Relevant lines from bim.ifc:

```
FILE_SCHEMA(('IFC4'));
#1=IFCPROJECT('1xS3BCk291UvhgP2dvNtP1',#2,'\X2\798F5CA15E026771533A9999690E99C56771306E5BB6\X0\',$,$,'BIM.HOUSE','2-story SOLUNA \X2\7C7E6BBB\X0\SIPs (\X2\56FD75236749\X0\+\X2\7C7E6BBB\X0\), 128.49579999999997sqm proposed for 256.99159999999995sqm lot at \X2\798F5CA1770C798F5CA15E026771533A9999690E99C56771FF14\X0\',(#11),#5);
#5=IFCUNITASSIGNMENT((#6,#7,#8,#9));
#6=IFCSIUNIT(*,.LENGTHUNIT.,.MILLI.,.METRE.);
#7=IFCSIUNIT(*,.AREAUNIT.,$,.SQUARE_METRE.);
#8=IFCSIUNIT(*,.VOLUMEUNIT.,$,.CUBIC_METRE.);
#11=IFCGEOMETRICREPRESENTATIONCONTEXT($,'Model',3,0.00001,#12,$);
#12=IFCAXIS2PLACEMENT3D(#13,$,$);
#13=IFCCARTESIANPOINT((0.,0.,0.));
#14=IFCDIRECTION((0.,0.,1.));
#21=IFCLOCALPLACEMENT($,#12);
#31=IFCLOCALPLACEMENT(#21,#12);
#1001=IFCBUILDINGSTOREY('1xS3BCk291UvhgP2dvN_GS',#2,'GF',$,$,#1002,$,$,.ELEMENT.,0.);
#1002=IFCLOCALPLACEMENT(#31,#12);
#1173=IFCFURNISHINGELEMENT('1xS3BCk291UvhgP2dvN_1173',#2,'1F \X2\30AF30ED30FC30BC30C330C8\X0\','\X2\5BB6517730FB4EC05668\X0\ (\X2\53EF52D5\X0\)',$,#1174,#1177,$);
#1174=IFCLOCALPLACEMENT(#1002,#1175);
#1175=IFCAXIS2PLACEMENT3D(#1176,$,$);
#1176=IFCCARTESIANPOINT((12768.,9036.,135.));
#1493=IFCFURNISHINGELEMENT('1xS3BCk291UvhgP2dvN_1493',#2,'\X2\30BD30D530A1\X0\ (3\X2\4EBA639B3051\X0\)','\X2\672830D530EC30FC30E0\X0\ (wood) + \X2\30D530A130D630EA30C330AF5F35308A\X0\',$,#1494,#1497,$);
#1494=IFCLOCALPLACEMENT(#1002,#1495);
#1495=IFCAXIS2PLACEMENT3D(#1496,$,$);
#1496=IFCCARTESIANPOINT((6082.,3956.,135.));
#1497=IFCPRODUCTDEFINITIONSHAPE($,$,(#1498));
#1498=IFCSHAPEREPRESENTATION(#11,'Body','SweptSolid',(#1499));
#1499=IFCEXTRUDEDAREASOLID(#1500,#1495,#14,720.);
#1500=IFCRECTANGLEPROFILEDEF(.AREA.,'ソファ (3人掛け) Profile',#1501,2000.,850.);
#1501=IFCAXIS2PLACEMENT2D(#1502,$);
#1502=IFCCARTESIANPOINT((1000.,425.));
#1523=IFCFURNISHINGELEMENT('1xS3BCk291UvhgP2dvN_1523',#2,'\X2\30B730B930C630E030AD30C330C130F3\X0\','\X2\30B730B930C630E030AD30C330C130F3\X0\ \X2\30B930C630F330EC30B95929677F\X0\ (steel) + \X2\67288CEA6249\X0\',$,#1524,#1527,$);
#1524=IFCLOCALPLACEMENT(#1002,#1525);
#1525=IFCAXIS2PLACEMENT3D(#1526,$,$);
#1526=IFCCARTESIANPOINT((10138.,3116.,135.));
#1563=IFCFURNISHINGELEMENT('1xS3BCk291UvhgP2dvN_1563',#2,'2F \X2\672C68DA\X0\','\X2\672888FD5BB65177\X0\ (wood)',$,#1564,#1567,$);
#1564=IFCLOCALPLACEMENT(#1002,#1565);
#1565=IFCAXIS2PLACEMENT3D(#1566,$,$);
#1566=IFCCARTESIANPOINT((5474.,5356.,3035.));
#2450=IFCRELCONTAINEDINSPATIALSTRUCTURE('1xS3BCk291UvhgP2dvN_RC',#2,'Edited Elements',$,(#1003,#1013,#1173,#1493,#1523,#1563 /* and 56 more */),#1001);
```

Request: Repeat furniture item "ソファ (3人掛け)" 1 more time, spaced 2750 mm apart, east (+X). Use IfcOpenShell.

```python
import numpy as np
import ifcopenshell
import ifcopenshell.api.geometry
import ifcopenshell.api.root
import ifcopenshell.util.element
import ifcopenshell.util.placement

model = ifcopenshell.open("bim.ifc")


def reuse_history(source, copy):
    """copy_class also copies each property set's owner history, people and application; keep the originals."""
    for rel in copy.IsDefinedBy:
        if rel.is_a("IfcRelDefinesByProperties") and (history := rel.RelatingPropertyDefinition.OwnerHistory):
            rel.RelatingPropertyDefinition.OwnerHistory = source.OwnerHistory
            ifcopenshell.util.element.remove_deep2(model, history)


source = model.by_guid("1xS3BCk291UvhgP2dvN_1493")
base = ifcopenshell.util.placement.get_local_placement(source.ObjectPlacement)
step = np.array([1.0, 0.0, 0.0]) * 2750.0

for i in range(1, 2):
    copy = ifcopenshell.api.root.copy_class(model, product=source)
    copy.Representation = ifcopenshell.util.element.copy_deep(
        model, source.Representation, exclude=["IfcGeometricRepresentationContext", "IfcRepresentationMap"]
    )
    reuse_history(source, copy)
    matrix = base.copy()
    matrix[:3, 3] += i * step
    print("added at", matrix[:3, 3].round(3) + 0.0)
    ifcopenshell.api.geometry.edit_object_placement(model, product=copy, matrix=matrix, is_si=False)

model.write("bim_v2.ifc")
```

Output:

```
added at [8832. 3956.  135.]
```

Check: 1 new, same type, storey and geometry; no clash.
